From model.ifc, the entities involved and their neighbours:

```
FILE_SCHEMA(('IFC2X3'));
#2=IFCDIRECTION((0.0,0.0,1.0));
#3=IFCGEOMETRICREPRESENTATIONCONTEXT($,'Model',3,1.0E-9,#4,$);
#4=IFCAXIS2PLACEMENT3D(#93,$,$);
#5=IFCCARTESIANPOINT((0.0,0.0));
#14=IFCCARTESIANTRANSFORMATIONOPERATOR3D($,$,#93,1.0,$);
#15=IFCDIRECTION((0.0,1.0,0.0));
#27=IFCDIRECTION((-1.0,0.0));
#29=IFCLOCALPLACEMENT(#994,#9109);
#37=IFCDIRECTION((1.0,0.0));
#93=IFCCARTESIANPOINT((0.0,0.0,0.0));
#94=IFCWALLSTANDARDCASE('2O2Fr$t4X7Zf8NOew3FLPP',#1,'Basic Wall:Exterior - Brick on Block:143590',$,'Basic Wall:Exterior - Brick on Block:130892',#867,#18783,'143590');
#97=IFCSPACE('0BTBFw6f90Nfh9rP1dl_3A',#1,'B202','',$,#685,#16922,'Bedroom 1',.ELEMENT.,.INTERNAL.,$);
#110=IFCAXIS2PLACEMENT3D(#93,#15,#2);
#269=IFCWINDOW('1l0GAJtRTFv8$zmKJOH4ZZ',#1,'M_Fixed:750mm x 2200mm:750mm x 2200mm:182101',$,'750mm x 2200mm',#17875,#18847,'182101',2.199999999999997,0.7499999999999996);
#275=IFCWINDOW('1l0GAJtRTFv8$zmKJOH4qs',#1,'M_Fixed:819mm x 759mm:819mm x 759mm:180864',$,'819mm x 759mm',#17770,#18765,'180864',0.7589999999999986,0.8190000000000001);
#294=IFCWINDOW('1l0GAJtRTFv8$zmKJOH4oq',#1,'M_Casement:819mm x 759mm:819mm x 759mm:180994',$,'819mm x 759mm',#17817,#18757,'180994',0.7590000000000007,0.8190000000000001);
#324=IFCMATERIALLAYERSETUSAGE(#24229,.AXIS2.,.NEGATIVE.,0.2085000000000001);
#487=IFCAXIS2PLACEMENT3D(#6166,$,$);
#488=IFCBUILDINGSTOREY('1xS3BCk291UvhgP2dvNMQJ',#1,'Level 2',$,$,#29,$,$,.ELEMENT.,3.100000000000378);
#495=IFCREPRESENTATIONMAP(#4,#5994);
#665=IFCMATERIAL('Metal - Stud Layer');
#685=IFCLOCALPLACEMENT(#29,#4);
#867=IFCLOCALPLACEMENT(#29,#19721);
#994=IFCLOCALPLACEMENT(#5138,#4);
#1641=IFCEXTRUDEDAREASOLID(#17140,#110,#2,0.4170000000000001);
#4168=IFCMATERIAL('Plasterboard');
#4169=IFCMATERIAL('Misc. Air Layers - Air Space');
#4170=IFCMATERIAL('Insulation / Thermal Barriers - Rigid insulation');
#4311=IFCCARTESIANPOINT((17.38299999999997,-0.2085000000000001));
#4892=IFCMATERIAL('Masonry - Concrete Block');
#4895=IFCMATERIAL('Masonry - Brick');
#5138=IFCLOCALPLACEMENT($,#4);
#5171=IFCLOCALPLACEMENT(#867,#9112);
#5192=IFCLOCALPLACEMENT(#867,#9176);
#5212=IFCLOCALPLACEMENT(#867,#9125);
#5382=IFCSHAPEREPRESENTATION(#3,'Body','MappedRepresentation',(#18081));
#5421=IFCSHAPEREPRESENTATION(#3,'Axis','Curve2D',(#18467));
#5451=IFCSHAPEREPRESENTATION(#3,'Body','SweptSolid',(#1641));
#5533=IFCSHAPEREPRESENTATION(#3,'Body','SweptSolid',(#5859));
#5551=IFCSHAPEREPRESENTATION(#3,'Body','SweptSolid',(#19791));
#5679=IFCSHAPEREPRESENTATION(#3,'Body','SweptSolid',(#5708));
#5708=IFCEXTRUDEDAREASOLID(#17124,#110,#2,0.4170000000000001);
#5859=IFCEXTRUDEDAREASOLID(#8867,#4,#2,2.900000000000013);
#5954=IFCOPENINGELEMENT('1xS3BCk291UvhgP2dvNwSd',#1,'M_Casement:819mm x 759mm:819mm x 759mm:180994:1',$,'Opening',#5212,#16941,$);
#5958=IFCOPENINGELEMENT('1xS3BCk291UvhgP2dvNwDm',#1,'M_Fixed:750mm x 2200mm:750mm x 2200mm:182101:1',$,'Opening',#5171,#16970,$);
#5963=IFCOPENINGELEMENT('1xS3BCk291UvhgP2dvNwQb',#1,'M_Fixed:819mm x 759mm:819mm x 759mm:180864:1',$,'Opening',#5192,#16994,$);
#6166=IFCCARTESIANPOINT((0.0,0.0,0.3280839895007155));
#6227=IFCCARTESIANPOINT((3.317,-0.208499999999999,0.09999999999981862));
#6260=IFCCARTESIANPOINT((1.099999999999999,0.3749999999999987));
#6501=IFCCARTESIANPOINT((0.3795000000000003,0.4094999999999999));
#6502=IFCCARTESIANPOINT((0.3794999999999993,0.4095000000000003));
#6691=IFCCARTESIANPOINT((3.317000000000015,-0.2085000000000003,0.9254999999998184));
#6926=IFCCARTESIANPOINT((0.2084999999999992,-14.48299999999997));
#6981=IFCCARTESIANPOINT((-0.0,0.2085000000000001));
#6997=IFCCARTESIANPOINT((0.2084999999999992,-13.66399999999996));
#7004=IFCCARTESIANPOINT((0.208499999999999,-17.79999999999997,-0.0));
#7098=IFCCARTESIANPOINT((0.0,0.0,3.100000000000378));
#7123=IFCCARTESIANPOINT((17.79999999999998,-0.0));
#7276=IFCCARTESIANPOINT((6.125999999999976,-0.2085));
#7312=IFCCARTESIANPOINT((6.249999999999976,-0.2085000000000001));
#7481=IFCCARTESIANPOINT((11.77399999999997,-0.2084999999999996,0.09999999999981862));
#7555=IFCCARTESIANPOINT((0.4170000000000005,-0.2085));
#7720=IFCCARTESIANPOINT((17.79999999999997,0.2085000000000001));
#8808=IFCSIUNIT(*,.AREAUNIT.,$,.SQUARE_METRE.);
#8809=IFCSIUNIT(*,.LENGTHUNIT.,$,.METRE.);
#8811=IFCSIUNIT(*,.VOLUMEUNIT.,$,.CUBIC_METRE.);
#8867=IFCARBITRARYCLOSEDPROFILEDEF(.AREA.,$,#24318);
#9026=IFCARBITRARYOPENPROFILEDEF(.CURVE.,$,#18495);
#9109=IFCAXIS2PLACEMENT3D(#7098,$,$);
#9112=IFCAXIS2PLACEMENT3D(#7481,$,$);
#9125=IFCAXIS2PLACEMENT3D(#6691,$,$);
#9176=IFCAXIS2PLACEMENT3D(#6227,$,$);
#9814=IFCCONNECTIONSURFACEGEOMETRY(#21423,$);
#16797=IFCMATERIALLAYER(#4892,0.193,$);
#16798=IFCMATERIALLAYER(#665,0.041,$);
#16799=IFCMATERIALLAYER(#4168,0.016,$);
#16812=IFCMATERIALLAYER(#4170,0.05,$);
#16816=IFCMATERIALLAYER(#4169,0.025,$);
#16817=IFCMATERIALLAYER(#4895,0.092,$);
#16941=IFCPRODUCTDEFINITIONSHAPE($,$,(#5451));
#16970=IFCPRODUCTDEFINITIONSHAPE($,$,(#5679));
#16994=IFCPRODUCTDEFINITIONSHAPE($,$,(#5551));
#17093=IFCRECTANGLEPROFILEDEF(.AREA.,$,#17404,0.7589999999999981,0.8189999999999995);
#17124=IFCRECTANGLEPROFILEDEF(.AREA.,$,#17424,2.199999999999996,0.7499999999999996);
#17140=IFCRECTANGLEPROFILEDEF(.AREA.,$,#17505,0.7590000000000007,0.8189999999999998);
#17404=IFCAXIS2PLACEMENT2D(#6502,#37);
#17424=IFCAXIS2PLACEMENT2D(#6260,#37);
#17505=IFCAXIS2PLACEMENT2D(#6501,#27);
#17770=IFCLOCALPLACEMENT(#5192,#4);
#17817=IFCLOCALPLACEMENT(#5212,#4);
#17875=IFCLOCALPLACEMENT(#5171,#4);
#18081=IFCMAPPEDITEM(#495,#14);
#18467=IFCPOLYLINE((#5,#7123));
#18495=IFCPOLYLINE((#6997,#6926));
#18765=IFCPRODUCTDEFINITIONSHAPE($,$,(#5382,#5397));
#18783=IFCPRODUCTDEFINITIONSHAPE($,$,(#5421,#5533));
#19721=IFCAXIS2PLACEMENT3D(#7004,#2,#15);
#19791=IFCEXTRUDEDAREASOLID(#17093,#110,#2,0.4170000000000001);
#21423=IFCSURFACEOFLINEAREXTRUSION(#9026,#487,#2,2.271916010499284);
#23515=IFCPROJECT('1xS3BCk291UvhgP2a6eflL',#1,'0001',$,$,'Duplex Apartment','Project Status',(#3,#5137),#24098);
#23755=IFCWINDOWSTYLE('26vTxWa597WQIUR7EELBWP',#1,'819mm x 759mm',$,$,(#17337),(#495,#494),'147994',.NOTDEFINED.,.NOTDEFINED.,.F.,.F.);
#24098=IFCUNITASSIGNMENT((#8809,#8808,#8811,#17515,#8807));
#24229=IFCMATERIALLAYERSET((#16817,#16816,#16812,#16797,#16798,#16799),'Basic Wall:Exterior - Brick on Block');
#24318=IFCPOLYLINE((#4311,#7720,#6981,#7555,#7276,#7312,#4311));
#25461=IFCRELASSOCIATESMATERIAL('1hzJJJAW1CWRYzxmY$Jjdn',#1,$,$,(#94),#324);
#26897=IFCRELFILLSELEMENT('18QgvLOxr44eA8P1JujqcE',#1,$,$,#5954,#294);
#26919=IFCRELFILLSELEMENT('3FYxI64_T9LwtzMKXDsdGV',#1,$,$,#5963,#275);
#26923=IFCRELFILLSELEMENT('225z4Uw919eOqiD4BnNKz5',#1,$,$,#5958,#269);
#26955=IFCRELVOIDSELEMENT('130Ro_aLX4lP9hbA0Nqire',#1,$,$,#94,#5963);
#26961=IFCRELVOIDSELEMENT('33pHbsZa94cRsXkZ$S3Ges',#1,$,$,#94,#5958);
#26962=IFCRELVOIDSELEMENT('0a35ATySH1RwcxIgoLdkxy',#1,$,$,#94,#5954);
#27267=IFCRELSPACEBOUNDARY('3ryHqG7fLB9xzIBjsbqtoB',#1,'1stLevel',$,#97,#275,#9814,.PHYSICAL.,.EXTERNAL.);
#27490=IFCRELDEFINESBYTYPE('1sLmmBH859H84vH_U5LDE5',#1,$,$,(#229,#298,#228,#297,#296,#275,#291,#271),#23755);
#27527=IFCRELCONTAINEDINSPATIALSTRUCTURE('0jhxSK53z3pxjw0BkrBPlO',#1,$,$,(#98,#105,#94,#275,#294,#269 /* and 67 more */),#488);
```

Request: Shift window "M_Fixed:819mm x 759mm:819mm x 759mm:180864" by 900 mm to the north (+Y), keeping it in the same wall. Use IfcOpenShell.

```python
import numpy as np
import ifcopenshell
import ifcopenshell.api.geometry
import ifcopenshell.util.placement
import ifcopenshell.util.unit

model = ifcopenshell.open("model.ifc")
unit_scale = ifcopenshell.util.unit.calculate_unit_scale(model)

window = model.by_guid("1l0GAJtRTFv8$zmKJOH4qs")
opening = window.FillsVoids[0].RelatingOpeningElement
wall = opening.VoidsElements[0].RelatingBuildingElement

wall_matrix = ifcopenshell.util.placement.get_local_placement(wall.ObjectPlacement)
shift = wall_matrix[:3, 0] * 0.9 / unit_scale
before = ifcopenshell.util.placement.get_local_placement(window.ObjectPlacement)[:3, 3].copy()

# The window is placed relative to its opening, so it follows when the opening moves.
matrix = ifcopenshell.util.placement.get_local_placement(opening.ObjectPlacement)
matrix[:3, 3] += shift
ifcopenshell.api.geometry.edit_object_placement(
    model, product=opening, matrix=matrix, is_si=False, should_transform_children=True
)

# Space boundary surfaces are stored in each space's coordinates; move them too.
for rel in window.ProvidesBoundaries:
    if not rel.ConnectionGeometry:
        continue
    surface = rel.ConnectionGeometry.SurfaceOnRelatingElement
    space_matrix = ifcopenshell.util.placement.get_local_placement(rel.RelatingSpace.ObjectPlacement)
    point = np.array(surface.Position.Location.Coordinates) + space_matrix[:3, :3].T @ shift
    surface.Position = model.createIfcAxis2Placement3D(
        model.createIfcCartesianPoint(point.tolist()), surface.Position.Axis, surface.Position.RefDirection
    )

after = ifcopenshell.util.placement.get_local_placement(window.ObjectPlacement)[:3, 3]
print("window moved by", (after - before).round(3) + 0.0)

model.write("model-out.ifc")
```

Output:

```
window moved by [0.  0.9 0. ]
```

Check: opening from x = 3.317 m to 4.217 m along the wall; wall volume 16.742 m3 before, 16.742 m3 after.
